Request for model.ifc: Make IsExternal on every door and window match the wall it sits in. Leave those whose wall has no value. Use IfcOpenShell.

First a look at what the model holds.

```python
import ifcopenshell
import ifcopenshell.util.element

model = ifcopenshell.open("model.ifc")
print(model.schema)
seen = {}
for e in model.by_type("IfcDoor") + model.by_type("IfcWindow"):
    if not e.FillsVoids:
        continue
    host = e.FillsVoids[0].RelatingOpeningElement.VoidsElements[0].RelatingBuildingElement
    own = ifcopenshell.util.element.get_pset(e, f"Pset_{e.is_a()[3:].removesuffix('StandardCase')}Common", "IsExternal")
    wall = ifcopenshell.util.element.get_pset(host, "Pset_WallCommon", "IsExternal")
    seen[e.is_a(), own, wall] = seen.get((e.is_a(), own, wall), 0) + 1
for (cls, own, wall), count in sorted(seen.items(), key=str):
    print(count, cls, "IsExternal:", own, "| host wall:", wall)
```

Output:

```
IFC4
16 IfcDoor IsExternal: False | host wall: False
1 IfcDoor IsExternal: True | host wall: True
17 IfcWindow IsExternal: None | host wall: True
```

```python
import ifcopenshell
import ifcopenshell.api.pset
import ifcopenshell.util.element

model = ifcopenshell.open("model.ifc")

count = 0
for ifc_class, pset_name in (("IfcDoor", "Pset_DoorCommon"), ("IfcWindow", "Pset_WindowCommon")):
    for e in model.by_type(ifc_class):
        if not e.FillsVoids:
            continue
        host = e.FillsVoids[0].RelatingOpeningElement.VoidsElements[0].RelatingBuildingElement
        external = ifcopenshell.util.element.get_pset(host, "Pset_WallCommon", "IsExternal")
        if external is None or ifcopenshell.util.element.get_pset(e, pset_name, "IsExternal") == external:
            continue
        pset = ifcopenshell.api.pset.add_pset(model, product=e, name=pset_name)
        ifcopenshell.api.pset.edit_pset(model, pset=pset, properties={"IsExternal": external})
        count += 1

print(count, "updated")

model.write("model_updated.ifc")
```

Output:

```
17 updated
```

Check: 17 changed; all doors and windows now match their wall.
